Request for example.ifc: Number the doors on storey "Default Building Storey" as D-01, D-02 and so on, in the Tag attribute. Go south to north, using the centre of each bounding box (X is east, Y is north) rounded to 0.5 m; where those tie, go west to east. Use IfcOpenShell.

First a look at what the model holds.

```python
import ifcopenshell
import ifcopenshell.util.element
import ifcopenshell.util.placement

model = ifcopenshell.open("example.ifc")
print(model.schema)
storey = next(s for s in model.by_type("IfcBuildingStorey") if s.Name == "Default Building Storey")
doors = [e for e in ifcopenshell.util.element.get_decomposition(storey) if e.is_a("IfcDoor")]
for e in sorted(doors, key=lambda e: e.id()):
    origin = ifcopenshell.util.placement.get_local_placement(e.ObjectPlacement)[:3, 3]
    print(e.id(), e.Tag, e.Name, origin.round(2) + 0.0, sep=" | ")
```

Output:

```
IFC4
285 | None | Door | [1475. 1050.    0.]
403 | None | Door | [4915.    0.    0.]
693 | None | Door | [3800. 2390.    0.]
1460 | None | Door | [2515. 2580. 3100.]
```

```python
import ifcopenshell
import ifcopenshell.geom
import ifcopenshell.util.element
import ifcopenshell.util.shape

model = ifcopenshell.open("example.ifc")
settings = ifcopenshell.geom.settings()
settings.set("use-world-coords", True)


def centre(element):
    shape = ifcopenshell.geom.create_shape(settings, element)
    return ifcopenshell.util.shape.get_bbox_centroid(shape.geometry)


storey = next(s for s in model.by_type("IfcBuildingStorey") if s.Name == "Default Building Storey")
doors = [e for e in ifcopenshell.util.element.get_decomposition(storey) if e.is_a("IfcDoor")]

# Insertion points can sit at a corner or the storey origin, so sort by the geometry (in metres).
centres = {e: centre(e) for e in doors}
doors.sort(key=lambda e: (round(centres[e][1] / 0.5), centres[e][0]))

for i, e in enumerate(doors, start=1):
    number = f"D-{i:02d}"
    e.Tag = number
    print(e.id(), number)

model.write("example_updated.ifc")
```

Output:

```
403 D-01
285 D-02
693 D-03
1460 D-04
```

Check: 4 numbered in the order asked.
